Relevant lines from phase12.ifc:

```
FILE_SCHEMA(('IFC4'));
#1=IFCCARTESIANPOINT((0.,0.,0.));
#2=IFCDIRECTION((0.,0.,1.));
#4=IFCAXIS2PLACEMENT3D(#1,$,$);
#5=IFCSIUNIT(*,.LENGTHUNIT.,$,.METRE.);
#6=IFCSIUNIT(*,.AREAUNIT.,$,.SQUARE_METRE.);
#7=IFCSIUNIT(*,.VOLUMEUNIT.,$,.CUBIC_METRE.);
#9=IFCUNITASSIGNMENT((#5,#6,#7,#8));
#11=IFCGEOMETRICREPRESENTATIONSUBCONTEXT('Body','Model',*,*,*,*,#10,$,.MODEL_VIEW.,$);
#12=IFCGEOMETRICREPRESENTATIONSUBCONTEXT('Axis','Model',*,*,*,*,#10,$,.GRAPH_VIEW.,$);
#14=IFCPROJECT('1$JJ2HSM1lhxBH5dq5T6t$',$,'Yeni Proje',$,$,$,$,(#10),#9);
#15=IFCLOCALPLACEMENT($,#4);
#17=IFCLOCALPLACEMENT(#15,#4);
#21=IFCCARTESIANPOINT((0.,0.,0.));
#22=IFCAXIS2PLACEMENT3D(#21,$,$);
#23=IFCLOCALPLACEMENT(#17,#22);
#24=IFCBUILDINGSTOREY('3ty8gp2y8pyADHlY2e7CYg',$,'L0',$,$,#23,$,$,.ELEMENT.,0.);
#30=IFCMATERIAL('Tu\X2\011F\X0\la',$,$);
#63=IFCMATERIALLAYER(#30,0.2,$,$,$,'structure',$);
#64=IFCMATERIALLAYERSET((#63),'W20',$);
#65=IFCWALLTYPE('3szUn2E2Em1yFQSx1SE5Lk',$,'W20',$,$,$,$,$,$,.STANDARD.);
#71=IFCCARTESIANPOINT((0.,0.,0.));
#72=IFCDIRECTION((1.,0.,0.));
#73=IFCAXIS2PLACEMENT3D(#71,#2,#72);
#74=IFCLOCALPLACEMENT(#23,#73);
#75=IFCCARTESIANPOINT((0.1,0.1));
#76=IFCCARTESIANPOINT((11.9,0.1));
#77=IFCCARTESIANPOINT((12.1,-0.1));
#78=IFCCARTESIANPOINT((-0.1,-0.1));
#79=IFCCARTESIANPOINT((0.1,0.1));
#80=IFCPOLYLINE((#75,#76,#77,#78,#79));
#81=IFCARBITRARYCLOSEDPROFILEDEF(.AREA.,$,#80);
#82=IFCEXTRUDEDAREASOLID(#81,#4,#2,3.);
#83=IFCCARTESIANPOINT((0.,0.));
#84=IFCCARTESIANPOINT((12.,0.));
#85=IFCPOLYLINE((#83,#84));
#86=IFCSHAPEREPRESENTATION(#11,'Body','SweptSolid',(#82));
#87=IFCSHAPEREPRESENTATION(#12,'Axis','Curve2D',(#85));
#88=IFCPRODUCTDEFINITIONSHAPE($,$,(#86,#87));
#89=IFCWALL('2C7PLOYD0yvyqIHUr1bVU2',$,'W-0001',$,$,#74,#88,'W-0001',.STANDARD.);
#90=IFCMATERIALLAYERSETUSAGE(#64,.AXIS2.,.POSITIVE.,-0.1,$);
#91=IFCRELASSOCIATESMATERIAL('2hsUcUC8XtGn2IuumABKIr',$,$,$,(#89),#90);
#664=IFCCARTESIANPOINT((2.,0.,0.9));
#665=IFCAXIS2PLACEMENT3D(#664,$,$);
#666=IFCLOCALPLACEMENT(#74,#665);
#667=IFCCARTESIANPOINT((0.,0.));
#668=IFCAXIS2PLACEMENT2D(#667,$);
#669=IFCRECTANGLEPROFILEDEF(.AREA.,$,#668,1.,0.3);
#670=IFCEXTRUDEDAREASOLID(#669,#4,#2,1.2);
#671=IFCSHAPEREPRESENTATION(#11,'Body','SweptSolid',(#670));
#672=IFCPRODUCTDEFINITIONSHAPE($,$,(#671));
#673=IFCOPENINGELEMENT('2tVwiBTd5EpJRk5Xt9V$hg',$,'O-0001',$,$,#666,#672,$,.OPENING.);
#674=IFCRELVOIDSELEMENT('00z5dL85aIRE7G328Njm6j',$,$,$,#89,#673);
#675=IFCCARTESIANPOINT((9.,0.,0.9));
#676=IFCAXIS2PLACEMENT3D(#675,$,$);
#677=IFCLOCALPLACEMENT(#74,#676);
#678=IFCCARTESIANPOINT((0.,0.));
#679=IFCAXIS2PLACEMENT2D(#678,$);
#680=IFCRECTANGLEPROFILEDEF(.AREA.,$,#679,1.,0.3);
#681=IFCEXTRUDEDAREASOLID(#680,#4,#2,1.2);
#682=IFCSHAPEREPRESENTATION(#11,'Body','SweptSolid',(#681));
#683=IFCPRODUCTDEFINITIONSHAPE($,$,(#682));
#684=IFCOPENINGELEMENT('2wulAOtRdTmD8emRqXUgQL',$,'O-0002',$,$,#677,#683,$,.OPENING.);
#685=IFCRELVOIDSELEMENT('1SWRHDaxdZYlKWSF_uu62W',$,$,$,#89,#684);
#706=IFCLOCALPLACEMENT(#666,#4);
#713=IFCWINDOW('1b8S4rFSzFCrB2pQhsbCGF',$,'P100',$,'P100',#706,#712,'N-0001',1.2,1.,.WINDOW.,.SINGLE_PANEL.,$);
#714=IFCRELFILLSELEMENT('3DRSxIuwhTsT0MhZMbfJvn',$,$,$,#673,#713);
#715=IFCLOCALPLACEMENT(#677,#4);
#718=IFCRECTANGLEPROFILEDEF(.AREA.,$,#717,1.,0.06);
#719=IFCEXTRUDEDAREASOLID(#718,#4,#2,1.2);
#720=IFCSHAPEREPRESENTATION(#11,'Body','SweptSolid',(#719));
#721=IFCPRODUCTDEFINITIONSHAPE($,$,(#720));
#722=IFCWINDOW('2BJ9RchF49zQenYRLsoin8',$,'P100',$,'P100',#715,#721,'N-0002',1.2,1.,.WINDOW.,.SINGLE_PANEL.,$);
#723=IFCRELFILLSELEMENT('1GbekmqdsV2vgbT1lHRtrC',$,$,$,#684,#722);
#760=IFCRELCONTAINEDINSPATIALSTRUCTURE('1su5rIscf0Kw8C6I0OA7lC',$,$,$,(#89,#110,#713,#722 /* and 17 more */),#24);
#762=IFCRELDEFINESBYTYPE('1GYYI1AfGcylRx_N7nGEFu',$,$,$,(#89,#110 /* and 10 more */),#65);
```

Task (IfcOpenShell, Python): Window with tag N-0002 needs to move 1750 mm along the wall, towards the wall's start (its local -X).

```python
import ifcopenshell
import ifcopenshell.api.geometry
import ifcopenshell.util.placement

model = ifcopenshell.open("phase12.ifc")

window = model.by_id(722)
opening = window.FillsVoids[0].RelatingOpeningElement
wall = opening.VoidsElements[0].RelatingBuildingElement

wall_matrix = ifcopenshell.util.placement.get_local_placement(wall.ObjectPlacement)
shift = wall_matrix[:3, 0] * -1.75
before = ifcopenshell.util.placement.get_local_placement(window.ObjectPlacement)[:3, 3].copy()

# The window is placed relative to its opening, so it follows when the opening moves.
matrix = ifcopenshell.util.placement.get_local_placement(opening.ObjectPlacement)
matrix[:3, 3] += shift
ifcopenshell.api.geometry.edit_object_placement(
    model, product=opening, matrix=matrix, is_si=False, should_transform_children=True
)

after = ifcopenshell.util.placement.get_local_placement(window.ObjectPlacement)[:3, 3]
print("window moved by", (after - before).round(3) + 0.0)

model.write("phase12_rev.ifc")
```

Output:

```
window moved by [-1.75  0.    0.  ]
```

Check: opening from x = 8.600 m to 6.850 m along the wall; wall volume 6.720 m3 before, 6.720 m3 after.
